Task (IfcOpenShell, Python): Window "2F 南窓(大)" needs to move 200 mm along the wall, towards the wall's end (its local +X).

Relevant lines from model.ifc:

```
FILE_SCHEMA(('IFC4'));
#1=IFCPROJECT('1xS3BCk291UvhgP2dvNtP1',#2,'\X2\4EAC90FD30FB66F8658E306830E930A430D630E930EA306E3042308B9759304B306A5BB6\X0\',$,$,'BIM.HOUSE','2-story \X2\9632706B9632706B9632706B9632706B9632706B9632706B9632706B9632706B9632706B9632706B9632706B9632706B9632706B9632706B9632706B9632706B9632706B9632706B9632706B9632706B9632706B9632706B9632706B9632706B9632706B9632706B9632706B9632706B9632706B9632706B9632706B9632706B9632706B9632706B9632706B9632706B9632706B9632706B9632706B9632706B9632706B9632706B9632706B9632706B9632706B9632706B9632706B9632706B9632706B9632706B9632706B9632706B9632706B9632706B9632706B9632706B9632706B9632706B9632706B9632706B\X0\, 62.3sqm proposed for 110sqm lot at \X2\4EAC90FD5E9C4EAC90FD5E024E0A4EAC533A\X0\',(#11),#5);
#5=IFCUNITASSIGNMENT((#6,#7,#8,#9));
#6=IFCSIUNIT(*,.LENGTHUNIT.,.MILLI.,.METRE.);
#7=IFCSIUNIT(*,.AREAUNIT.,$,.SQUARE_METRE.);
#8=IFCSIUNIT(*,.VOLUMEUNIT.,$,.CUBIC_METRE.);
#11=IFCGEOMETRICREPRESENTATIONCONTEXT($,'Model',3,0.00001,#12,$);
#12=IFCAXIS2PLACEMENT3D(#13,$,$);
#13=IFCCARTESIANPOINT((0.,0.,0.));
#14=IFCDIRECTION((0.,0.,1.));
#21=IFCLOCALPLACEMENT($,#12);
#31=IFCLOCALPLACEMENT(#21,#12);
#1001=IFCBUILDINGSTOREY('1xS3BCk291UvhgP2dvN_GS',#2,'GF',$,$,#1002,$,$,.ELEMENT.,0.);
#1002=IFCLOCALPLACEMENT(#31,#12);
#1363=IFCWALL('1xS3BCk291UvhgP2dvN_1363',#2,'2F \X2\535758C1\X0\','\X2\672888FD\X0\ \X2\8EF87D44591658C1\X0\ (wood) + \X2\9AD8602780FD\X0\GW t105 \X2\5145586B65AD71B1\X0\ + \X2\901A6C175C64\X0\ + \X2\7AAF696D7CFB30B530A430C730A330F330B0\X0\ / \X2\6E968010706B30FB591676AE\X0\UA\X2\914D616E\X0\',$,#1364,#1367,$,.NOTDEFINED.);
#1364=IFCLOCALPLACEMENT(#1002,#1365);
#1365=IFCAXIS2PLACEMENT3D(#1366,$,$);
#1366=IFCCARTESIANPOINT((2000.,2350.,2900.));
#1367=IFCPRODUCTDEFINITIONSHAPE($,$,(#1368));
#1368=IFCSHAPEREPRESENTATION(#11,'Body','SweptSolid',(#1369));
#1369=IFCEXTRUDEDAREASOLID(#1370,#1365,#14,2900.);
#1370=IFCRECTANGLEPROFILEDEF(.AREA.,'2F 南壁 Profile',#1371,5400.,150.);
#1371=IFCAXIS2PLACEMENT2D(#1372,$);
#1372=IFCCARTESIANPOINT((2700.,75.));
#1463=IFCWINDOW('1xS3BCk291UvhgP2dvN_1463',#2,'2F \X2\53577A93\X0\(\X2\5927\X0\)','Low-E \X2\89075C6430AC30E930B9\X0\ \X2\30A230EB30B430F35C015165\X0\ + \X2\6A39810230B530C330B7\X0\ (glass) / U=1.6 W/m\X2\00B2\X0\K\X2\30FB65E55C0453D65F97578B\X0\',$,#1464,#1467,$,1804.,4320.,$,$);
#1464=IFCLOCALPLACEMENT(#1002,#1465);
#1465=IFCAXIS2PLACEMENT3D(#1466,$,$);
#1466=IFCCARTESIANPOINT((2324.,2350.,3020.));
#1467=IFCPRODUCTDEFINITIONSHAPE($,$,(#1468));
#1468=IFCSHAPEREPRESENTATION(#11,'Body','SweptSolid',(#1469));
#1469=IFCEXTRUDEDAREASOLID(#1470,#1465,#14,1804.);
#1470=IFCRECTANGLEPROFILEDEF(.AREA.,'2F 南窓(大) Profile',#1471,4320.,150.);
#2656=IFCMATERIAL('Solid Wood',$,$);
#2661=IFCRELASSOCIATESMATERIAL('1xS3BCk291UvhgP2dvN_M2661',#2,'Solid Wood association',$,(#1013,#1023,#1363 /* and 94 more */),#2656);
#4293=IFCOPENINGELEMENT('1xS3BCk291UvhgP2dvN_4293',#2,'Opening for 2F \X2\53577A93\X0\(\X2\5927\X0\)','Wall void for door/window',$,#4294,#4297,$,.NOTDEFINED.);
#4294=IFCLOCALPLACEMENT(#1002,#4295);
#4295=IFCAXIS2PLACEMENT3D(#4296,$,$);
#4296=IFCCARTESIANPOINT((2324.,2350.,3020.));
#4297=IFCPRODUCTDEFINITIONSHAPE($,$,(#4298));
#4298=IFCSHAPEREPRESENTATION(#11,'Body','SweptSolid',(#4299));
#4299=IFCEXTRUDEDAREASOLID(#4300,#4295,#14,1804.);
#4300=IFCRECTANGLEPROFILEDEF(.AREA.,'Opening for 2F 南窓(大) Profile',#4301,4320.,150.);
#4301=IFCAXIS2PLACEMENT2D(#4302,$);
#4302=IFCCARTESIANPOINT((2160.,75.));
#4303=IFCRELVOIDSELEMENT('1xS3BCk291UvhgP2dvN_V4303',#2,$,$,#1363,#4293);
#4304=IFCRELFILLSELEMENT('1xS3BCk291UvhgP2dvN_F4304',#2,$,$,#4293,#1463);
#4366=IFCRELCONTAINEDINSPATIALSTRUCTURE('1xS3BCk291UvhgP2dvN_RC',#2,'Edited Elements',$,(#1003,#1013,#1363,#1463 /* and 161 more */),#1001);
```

```python
import ifcopenshell
import ifcopenshell.api.geometry
import ifcopenshell.util.placement
import ifcopenshell.util.unit

model = ifcopenshell.open("model.ifc")
unit_scale = ifcopenshell.util.unit.calculate_unit_scale(model)

window = model.by_guid("1xS3BCk291UvhgP2dvN_1463")
opening = window.FillsVoids[0].RelatingOpeningElement
wall = opening.VoidsElements[0].RelatingBuildingElement

wall_matrix = ifcopenshell.util.placement.get_local_placement(wall.ObjectPlacement)
shift = wall_matrix[:3, 0] * 0.2 / unit_scale
before = ifcopenshell.util.placement.get_local_placement(window.ObjectPlacement)[:3, 3].copy()

# The window is not placed relative to its opening, so move both.
for product in (opening, window):
    matrix = ifcopenshell.util.placement.get_local_placement(product.ObjectPlacement)
    matrix[:3, 3] += shift
    ifcopenshell.api.geometry.edit_object_placement(model, product=product, matrix=matrix, is_si=False)

after = ifcopenshell.util.placement.get_local_placement(window.ObjectPlacement)[:3, 3]
print("window moved by", (after - before).round(3) + 0.0)

model.write("model_edited.ifc")
```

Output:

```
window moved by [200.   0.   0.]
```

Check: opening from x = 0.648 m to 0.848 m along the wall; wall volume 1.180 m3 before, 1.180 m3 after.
